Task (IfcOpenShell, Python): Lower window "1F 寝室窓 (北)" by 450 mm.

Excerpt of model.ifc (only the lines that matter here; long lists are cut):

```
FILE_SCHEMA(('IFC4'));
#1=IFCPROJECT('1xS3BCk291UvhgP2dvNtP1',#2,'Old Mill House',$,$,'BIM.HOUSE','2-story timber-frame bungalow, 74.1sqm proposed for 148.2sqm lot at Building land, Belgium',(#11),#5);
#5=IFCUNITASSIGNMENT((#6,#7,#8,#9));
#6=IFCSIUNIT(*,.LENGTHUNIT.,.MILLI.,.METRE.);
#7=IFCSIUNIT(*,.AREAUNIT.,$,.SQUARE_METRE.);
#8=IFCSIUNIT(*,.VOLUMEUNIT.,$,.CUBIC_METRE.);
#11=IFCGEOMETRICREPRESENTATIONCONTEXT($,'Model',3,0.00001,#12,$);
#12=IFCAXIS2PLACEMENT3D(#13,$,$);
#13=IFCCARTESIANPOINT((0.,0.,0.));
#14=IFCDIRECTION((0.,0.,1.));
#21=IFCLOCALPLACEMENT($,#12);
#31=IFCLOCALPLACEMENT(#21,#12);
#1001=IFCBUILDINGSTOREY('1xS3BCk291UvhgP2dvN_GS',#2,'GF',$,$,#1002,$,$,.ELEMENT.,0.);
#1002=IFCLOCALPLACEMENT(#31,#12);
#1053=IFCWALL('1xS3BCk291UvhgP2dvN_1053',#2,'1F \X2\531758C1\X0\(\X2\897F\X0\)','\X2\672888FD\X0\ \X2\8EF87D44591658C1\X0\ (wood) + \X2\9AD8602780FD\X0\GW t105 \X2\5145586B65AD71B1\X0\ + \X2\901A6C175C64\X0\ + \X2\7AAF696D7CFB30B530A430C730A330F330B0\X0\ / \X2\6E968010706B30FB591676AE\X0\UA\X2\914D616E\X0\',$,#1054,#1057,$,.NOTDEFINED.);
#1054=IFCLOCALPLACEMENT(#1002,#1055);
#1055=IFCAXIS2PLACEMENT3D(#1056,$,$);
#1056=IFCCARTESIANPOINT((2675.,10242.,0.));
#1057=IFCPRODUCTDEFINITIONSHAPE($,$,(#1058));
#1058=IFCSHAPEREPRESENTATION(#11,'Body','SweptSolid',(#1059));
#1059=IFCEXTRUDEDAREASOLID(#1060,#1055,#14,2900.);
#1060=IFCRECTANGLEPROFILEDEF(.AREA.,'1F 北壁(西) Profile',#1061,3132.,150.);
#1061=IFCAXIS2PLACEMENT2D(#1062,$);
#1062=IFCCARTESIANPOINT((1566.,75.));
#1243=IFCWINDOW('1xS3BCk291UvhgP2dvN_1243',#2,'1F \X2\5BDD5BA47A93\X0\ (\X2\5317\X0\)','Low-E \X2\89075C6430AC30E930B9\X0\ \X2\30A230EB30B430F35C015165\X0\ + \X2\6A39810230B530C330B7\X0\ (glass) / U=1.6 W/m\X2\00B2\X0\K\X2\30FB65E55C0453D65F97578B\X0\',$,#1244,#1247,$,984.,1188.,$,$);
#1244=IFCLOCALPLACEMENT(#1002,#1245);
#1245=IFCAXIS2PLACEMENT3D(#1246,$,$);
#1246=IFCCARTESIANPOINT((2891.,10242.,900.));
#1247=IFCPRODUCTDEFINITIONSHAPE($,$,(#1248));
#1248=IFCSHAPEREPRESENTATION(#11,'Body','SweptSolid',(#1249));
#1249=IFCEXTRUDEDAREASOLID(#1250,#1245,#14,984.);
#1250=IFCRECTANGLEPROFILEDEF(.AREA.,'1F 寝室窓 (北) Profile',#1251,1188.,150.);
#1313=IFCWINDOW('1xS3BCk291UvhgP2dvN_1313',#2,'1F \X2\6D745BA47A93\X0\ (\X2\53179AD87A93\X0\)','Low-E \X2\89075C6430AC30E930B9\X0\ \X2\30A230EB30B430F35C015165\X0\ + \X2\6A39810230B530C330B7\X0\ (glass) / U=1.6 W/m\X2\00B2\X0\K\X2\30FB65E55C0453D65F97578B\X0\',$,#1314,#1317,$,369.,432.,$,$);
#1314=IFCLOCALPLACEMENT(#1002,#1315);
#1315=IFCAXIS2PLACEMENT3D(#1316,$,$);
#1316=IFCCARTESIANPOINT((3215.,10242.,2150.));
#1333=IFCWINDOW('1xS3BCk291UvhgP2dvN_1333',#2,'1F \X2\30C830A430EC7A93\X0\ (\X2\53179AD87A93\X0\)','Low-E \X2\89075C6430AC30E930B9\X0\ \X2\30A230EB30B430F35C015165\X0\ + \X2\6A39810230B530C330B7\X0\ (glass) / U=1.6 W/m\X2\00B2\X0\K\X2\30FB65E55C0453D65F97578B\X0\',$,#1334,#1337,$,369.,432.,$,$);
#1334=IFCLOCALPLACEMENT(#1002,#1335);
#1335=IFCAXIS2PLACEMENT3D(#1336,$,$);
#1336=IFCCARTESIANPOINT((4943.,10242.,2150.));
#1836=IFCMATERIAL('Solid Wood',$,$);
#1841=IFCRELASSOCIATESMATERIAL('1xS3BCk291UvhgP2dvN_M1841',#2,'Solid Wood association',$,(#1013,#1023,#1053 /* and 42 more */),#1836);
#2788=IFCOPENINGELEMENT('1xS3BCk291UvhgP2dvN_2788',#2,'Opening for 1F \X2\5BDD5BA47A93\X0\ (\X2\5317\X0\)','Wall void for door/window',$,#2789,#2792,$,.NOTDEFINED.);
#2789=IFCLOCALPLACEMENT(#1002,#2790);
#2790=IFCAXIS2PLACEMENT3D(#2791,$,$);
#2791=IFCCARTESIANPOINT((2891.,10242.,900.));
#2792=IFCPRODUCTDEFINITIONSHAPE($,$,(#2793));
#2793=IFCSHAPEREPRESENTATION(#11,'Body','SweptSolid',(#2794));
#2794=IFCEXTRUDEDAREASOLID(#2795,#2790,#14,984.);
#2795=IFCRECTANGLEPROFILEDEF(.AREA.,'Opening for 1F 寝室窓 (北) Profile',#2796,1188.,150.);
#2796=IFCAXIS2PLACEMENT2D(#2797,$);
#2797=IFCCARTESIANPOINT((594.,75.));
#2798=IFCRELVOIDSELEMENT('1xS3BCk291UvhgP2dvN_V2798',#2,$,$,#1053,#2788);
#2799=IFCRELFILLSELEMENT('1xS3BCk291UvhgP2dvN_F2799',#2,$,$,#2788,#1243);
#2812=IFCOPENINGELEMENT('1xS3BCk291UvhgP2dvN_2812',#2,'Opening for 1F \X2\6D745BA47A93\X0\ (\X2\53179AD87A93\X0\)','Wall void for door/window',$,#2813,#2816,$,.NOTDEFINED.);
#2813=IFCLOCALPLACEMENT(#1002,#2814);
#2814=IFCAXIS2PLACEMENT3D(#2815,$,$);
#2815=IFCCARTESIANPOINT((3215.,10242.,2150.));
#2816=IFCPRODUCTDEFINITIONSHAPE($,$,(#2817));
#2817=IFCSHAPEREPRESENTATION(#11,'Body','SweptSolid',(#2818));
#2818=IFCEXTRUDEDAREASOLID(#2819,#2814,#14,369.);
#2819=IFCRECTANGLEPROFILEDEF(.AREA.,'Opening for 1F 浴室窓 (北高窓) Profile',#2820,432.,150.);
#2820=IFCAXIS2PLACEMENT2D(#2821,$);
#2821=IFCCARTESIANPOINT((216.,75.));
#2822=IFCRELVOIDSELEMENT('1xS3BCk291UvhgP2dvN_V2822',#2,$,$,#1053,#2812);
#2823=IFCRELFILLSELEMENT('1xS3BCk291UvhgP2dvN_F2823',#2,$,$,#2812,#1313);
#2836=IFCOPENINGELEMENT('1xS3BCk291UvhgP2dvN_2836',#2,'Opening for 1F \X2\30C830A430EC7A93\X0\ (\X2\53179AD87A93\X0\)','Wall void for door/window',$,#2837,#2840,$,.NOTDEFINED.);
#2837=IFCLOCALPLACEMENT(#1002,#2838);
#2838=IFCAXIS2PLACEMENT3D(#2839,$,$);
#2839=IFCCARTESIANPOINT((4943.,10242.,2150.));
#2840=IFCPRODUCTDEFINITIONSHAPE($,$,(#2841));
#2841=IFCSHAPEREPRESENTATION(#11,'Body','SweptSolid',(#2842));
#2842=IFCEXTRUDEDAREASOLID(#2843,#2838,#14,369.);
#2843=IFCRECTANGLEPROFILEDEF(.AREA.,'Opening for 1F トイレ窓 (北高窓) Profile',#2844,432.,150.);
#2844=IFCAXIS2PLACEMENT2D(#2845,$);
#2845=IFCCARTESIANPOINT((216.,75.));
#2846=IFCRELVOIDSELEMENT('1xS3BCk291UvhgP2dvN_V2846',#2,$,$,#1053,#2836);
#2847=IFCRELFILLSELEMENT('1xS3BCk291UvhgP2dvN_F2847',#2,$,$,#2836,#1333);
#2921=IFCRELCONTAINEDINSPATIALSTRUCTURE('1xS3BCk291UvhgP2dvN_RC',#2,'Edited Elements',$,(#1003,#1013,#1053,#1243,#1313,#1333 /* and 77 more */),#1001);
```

```python
import numpy as np
import ifcopenshell
import ifcopenshell.api.geometry
import ifcopenshell.util.placement
import ifcopenshell.util.unit

model = ifcopenshell.open("model.ifc")
unit_scale = ifcopenshell.util.unit.calculate_unit_scale(model)

window = model.by_guid("1xS3BCk291UvhgP2dvN_1243")
opening = window.FillsVoids[0].RelatingOpeningElement
dz = -0.45 / unit_scale

shift = np.array([0.0, 0.0, dz])
# The window is not placed relative to its opening, so move both.
for product in (opening, window):
    matrix = ifcopenshell.util.placement.get_local_placement(product.ObjectPlacement)
    matrix[:3, 3] += shift
    ifcopenshell.api.geometry.edit_object_placement(model, product=product, matrix=matrix, is_si=False)

print(f"moved by {dz * unit_scale:+.3f} m")

model.write("model_rev.ifc")
```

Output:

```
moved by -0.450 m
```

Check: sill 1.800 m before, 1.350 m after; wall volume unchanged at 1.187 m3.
